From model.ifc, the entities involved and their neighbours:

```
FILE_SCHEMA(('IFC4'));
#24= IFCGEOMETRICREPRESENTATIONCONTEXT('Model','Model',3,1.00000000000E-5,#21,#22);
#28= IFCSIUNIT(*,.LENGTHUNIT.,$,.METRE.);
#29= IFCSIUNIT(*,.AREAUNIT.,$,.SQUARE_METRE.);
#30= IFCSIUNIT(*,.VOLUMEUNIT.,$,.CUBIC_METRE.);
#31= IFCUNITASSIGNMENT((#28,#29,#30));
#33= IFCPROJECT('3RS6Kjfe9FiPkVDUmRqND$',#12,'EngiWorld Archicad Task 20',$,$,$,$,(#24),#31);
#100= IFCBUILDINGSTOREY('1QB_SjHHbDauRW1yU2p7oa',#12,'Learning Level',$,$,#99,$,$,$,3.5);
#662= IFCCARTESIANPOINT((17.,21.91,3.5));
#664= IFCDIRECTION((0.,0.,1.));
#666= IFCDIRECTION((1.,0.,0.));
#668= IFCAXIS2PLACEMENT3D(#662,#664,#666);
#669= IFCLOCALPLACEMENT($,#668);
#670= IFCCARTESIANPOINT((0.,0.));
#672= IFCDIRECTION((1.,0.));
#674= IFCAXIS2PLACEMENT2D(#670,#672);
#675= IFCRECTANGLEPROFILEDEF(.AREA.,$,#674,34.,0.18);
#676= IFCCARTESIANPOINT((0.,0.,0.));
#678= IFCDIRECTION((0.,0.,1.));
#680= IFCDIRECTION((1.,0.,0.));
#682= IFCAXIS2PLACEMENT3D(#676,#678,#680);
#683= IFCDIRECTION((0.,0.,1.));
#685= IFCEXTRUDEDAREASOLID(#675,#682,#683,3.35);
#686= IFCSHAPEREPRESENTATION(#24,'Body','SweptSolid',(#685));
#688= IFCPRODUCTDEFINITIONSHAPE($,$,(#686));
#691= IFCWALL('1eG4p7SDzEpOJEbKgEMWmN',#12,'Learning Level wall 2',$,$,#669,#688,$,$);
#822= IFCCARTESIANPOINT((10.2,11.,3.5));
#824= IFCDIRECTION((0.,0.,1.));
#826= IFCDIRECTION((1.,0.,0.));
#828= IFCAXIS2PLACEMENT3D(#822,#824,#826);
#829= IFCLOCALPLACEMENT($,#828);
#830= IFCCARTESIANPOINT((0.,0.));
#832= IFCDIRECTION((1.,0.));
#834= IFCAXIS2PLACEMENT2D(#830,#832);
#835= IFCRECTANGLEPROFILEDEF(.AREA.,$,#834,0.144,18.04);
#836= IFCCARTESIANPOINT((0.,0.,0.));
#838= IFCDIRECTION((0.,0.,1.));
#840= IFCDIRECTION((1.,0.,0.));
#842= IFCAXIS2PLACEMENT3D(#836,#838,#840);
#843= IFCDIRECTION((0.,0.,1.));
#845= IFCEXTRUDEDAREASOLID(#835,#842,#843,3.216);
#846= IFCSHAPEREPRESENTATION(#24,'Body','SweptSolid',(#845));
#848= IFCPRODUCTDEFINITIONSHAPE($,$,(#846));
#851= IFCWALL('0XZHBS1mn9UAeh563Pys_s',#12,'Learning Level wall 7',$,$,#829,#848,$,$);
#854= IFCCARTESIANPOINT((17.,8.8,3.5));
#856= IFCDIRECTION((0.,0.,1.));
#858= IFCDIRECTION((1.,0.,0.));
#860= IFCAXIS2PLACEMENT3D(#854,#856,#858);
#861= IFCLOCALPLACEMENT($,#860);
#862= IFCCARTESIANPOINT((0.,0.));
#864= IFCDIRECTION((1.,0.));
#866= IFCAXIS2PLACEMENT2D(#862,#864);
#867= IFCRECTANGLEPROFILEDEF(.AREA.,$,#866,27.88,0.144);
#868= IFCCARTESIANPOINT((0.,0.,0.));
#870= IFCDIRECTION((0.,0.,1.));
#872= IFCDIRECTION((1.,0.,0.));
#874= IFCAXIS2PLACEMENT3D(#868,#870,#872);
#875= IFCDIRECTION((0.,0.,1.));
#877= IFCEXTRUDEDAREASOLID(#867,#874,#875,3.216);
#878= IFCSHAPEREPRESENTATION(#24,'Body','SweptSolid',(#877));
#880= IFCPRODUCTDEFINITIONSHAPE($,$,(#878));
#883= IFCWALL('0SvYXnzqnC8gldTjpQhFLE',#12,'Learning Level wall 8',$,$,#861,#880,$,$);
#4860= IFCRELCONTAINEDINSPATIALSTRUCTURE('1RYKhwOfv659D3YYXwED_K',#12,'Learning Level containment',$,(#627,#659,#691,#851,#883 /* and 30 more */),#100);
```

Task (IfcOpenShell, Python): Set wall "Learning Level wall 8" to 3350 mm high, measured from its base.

```python
import ifcopenshell
import ifcopenshell.geom
import ifcopenshell.util.shape

model = ifcopenshell.open("model.ifc")
settings = ifcopenshell.geom.settings()


def volume(element):
    """Net volume in cubic metres, openings subtracted."""
    shape = ifcopenshell.geom.create_shape(settings, element)
    return ifcopenshell.util.shape.get_volume(shape.geometry)


wall = model.by_guid("0SvYXnzqnC8gldTjpQhFLE")
before = volume(wall)

body = next(r for r in wall.Representation.Representations if r.RepresentationIdentifier == "Body")
solid = body.Items[0]
old_height = solid.Depth
solid.Depth = 3.35
after = volume(wall)

print(f"height {old_height:g} -> {solid.Depth:g}, volume {before:.3f} -> {after:.3f} m3")

model.write("model_updated.ifc")
```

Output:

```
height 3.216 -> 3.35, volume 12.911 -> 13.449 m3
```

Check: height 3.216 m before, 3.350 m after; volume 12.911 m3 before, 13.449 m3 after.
